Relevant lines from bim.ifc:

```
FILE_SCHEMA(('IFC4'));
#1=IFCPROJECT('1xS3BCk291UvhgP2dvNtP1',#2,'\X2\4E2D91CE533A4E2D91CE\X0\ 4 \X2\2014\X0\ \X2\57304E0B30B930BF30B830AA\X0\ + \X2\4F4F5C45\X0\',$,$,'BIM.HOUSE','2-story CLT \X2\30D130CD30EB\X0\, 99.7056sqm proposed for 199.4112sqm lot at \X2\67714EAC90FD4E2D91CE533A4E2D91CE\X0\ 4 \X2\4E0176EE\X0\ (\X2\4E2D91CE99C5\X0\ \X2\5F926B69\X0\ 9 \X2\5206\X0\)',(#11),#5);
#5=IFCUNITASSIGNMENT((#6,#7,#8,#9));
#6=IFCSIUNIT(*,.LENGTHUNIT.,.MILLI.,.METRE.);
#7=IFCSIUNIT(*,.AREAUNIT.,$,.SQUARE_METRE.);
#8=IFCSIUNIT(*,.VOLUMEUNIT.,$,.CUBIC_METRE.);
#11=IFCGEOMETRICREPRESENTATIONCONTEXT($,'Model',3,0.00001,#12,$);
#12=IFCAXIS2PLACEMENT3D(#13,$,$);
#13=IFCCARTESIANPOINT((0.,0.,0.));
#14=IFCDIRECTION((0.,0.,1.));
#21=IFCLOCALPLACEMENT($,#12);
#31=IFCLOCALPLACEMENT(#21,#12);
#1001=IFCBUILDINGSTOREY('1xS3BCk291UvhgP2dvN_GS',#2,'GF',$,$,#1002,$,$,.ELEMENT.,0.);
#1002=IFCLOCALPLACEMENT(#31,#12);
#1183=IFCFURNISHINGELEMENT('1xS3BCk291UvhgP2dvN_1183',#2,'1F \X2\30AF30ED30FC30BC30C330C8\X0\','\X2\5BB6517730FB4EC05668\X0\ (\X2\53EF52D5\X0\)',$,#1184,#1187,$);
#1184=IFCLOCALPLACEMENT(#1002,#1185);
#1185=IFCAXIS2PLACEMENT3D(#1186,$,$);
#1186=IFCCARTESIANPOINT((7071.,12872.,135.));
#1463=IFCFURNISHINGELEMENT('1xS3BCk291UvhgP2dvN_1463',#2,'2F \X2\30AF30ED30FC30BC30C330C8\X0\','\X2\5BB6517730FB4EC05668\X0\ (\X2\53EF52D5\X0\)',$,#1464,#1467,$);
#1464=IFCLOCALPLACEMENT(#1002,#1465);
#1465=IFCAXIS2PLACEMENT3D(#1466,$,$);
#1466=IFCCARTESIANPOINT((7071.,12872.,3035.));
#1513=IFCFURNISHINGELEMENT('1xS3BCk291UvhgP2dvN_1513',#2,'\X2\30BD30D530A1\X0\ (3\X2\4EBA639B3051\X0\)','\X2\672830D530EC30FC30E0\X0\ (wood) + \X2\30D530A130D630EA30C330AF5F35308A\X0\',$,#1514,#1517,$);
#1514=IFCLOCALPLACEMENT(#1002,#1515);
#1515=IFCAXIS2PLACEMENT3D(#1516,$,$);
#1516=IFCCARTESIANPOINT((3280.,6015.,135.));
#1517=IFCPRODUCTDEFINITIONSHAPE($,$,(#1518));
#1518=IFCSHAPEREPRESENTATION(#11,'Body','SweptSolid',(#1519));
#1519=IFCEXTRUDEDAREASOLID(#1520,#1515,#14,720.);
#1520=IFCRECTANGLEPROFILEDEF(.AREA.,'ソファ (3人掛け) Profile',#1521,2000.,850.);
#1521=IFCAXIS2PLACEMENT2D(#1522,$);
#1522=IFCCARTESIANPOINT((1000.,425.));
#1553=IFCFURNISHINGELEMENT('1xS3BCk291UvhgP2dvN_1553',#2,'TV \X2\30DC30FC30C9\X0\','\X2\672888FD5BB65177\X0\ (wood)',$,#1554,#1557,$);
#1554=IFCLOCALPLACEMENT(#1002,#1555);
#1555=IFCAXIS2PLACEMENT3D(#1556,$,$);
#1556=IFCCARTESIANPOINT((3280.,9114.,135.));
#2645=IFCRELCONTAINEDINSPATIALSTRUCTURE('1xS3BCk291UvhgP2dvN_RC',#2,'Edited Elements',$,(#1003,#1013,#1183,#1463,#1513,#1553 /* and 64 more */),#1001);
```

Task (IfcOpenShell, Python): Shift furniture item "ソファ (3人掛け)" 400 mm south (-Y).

```python
import ifcopenshell
import ifcopenshell.api.geometry
import ifcopenshell.util.placement
import ifcopenshell.util.unit

model = ifcopenshell.open("bim.ifc")
unit_scale = ifcopenshell.util.unit.calculate_unit_scale(model)

item = model.by_guid("1xS3BCk291UvhgP2dvN_1513")
matrix = ifcopenshell.util.placement.get_local_placement(item.ObjectPlacement)
matrix[1, 3] -= 0.4 / unit_scale
ifcopenshell.api.geometry.edit_object_placement(model, product=item, matrix=matrix, is_si=False)

print(ifcopenshell.util.placement.get_local_placement(item.ObjectPlacement).round(3) + 0.0)

model.write("bim_edited.ifc")
```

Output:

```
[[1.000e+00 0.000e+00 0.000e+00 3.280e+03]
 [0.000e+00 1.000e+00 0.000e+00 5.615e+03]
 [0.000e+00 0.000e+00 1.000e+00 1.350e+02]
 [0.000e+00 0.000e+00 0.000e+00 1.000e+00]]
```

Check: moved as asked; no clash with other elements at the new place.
